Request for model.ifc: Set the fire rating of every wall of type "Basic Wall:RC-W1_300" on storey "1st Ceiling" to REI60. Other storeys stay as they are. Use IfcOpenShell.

First a look at what the model holds.

```python
import ifcopenshell
import ifcopenshell.util.element

model = ifcopenshell.open("model.ifc")
print(model.schema)
storey = next(s for s in model.by_type("IfcBuildingStorey") if s.Name == "1st Ceiling")
walls = [e for e in ifcopenshell.util.element.get_decomposition(storey) if e.is_a("IfcWall")]
seen = {}
for e in walls:
    element_type = ifcopenshell.util.element.get_type(e)
    key = (element_type.Name if element_type != e and element_type else None, ifcopenshell.util.element.get_pset(e, "Pset_WallCommon", "FireRating"))
    seen[key] = seen.get(key, 0) + 1
for (name, value), count in sorted(seen.items(), key=str):
    print(count, "x", name, "|", value)
```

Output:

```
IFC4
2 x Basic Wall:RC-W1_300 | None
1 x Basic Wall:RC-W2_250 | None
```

```python
import ifcopenshell
import ifcopenshell.api.pset
import ifcopenshell.util.element

model = ifcopenshell.open("model.ifc")

storey = next(s for s in model.by_type("IfcBuildingStorey") if s.Name == "1st Ceiling")
walls = [e for e in ifcopenshell.util.element.get_decomposition(storey) if e.is_a("IfcWall")]

count = 0
for e in walls:
    element_type = ifcopenshell.util.element.get_type(e)
    if element_type in (None, e) or element_type.Name != "Basic Wall:RC-W1_300":
        continue
    # add_pset returns the element's existing set when there is one.
    pset = ifcopenshell.api.pset.add_pset(model, product=e, name="Pset_WallCommon")
    ifcopenshell.api.pset.edit_pset(model, pset=pset, properties={"FireRating": "REI60"})
    count += 1

print(count, "walls updated")

model.write("model_rev.ifc")
```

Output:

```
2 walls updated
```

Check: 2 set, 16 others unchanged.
